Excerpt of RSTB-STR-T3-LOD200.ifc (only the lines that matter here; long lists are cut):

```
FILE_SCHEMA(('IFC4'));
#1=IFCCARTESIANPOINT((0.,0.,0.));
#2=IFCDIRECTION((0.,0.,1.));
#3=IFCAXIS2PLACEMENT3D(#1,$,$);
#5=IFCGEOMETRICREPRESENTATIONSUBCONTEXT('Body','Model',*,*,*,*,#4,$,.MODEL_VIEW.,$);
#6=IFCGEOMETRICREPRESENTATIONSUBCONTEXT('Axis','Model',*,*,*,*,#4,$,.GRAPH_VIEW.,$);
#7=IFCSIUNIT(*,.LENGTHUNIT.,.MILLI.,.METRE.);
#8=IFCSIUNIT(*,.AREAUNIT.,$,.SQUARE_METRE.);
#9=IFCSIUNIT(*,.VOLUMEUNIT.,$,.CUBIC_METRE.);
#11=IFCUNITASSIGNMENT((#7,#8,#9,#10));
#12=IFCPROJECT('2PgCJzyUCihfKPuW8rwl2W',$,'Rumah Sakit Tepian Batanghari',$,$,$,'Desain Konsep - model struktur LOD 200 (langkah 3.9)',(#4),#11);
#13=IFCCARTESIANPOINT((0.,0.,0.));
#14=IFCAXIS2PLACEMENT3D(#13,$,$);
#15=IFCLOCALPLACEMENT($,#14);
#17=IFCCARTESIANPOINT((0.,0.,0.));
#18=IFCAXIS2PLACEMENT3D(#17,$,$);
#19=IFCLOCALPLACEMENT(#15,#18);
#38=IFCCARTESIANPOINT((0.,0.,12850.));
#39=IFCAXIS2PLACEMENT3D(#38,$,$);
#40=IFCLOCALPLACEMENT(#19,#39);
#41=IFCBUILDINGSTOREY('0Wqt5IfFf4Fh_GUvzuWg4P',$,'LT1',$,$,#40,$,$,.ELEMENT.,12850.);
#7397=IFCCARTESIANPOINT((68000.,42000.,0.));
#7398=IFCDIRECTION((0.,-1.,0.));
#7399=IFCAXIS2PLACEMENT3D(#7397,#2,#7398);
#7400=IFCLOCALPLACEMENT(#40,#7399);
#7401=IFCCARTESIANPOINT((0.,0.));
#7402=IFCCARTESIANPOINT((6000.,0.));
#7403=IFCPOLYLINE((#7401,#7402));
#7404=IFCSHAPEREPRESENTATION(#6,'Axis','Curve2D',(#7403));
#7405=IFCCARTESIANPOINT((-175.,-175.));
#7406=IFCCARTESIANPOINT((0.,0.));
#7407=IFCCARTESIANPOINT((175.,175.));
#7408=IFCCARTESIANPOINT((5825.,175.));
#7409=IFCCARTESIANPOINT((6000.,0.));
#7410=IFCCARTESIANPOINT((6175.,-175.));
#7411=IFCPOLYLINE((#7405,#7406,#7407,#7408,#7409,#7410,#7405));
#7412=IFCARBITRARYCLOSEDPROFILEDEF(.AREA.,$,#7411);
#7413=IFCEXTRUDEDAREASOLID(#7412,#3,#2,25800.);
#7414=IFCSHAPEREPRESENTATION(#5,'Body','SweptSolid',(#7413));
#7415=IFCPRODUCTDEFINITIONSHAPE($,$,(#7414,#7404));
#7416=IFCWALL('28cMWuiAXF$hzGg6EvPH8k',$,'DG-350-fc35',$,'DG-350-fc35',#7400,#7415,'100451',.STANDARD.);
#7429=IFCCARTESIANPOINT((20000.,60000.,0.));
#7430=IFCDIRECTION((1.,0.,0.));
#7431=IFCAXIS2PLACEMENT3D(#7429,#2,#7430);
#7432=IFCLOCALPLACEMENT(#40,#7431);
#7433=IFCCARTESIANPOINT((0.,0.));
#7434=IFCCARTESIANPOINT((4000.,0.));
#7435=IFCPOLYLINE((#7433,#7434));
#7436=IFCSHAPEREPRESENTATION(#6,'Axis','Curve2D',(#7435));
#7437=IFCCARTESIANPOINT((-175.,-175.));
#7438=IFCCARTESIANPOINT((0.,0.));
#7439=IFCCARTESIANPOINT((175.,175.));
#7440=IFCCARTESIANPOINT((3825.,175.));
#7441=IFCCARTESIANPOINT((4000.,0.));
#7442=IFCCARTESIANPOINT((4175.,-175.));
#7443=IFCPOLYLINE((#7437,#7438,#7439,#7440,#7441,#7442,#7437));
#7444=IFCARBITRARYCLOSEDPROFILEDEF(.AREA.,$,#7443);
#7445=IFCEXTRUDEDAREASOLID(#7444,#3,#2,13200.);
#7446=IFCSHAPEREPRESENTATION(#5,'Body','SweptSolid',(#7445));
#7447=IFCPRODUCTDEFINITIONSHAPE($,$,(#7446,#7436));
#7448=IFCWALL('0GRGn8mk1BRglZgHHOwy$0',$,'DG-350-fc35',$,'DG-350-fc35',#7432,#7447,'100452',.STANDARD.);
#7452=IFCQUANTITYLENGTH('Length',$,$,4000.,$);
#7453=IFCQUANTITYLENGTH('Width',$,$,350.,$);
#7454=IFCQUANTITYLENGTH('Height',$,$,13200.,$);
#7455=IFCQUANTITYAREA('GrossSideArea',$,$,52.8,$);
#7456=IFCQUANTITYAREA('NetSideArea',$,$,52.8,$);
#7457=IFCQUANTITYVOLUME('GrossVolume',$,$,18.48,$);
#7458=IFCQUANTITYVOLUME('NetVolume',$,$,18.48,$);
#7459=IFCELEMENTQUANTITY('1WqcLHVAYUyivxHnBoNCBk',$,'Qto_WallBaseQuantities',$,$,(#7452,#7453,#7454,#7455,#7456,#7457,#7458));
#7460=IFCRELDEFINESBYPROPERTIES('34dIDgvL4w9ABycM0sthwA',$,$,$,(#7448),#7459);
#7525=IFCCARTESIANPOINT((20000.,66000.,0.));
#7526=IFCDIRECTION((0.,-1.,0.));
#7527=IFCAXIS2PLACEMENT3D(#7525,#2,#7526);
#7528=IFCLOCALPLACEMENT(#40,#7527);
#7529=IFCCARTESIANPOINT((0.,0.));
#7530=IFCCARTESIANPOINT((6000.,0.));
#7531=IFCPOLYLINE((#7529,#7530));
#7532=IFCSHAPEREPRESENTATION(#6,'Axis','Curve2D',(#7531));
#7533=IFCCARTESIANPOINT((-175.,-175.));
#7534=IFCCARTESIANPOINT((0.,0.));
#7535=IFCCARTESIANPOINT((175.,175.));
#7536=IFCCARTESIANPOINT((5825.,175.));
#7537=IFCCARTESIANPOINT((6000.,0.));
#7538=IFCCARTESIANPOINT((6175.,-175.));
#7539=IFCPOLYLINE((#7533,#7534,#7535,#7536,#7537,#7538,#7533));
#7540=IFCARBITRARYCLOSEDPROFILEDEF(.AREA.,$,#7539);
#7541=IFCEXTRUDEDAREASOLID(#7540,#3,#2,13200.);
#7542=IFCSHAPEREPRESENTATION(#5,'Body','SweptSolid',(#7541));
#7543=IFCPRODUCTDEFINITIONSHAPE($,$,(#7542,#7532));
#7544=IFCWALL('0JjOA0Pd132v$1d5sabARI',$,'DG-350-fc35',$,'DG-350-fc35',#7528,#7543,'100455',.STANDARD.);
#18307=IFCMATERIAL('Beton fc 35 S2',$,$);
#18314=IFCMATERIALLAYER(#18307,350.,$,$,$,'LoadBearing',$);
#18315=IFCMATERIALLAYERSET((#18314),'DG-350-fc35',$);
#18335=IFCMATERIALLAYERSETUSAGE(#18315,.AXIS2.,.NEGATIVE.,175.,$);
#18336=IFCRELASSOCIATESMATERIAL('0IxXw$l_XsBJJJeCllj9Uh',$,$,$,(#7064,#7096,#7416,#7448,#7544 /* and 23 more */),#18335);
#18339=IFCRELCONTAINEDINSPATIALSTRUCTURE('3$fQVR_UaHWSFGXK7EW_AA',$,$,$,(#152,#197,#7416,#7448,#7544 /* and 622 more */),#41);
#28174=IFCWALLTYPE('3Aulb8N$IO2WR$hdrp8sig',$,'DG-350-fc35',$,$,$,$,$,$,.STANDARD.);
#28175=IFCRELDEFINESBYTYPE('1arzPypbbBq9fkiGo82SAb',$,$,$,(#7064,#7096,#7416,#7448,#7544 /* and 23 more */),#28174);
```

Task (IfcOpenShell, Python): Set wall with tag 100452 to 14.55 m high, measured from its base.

```python
import ifcopenshell
import ifcopenshell.api.pset
import ifcopenshell.geom
import ifcopenshell.util.element
import ifcopenshell.util.representation
import ifcopenshell.util.shape
import ifcopenshell.util.unit

model = ifcopenshell.open("RSTB-STR-T3-LOD200.ifc")
unit_scale = ifcopenshell.util.unit.calculate_unit_scale(model)
area_scale = ifcopenshell.util.unit.calculate_unit_scale(model, "AREAUNIT")
volume_scale = ifcopenshell.util.unit.calculate_unit_scale(model, "VOLUMEUNIT")
settings = ifcopenshell.geom.settings()


def volume(element):
    """Net volume in cubic metres, openings subtracted."""
    shape = ifcopenshell.geom.create_shape(settings, element)
    return ifcopenshell.util.shape.get_volume(shape.geometry)


wall = model.by_guid("0GRGn8mk1BRglZgHHOwy$0")
before = volume(wall)

body = ifcopenshell.util.representation.get_representation(wall, "Model", "Body")
solid = body.Items[0]
old_height = solid.Depth
solid.Depth = 14.55 / unit_scale
after = volume(wall)
thickness = 0.35  # wall thickness in metres

# Update the stored height, areas and volumes.
qto = model.by_id(ifcopenshell.util.element.get_pset(wall, "Qto_WallBaseQuantities", should_inherit=False)["id"])
ifcopenshell.api.pset.edit_qto(model, qto=qto, properties={
    "Height": solid.Depth,
    "GrossSideArea": ifcopenshell.util.element.get_pset(wall, "Qto_WallBaseQuantities", "GrossSideArea") * solid.Depth / old_height,
    "NetSideArea": after / thickness / area_scale,
    "GrossVolume": ifcopenshell.util.element.get_pset(wall, "Qto_WallBaseQuantities", "GrossVolume") * solid.Depth / old_height,
    "NetVolume": after / volume_scale,
})

print(f"height {old_height:g} -> {solid.Depth:g}, volume {before:.3f} -> {after:.3f} m3")

model.write("RSTB-STR-T3-LOD200_v2.ifc")
```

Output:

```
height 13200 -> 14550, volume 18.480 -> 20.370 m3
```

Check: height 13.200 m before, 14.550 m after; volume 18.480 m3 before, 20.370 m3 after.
